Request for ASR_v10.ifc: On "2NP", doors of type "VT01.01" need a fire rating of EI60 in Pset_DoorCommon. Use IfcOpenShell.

First a look at what the model holds.

```python
import ifcopenshell
import ifcopenshell.util.element

model = ifcopenshell.open("ASR_v10.ifc")
print(model.schema)
storey = next(s for s in model.by_type("IfcBuildingStorey") if s.Name == "2NP")
doors = [e for e in ifcopenshell.util.element.get_decomposition(storey) if e.is_a("IfcDoor")]
seen = {}
for e in doors:
    element_type = ifcopenshell.util.element.get_type(e)
    key = (element_type.Name if element_type != e and element_type else None, ifcopenshell.util.element.get_pset(e, "Pset_DoorCommon", "FireRating"))
    seen[key] = seen.get(key, 0) + 1
for (name, value), count in sorted(seen.items(), key=str):
    print(count, "x", name, "|", value)
```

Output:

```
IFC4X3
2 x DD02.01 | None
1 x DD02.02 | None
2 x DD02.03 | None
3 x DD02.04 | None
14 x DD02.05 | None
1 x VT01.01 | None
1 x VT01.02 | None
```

```python
import ifcopenshell
import ifcopenshell.api.pset
import ifcopenshell.util.element

model = ifcopenshell.open("ASR_v10.ifc")

storey = next(s for s in model.by_type("IfcBuildingStorey") if s.Name == "2NP")
doors = [e for e in ifcopenshell.util.element.get_decomposition(storey) if e.is_a("IfcDoor")]

count = 0
for e in doors:
    element_type = ifcopenshell.util.element.get_type(e)
    if element_type in (None, e) or element_type.Name != "VT01.01":
        continue
    # add_pset returns the element's existing set when there is one.
    pset = ifcopenshell.api.pset.add_pset(model, product=e, name="Pset_DoorCommon")
    ifcopenshell.api.pset.edit_pset(model, pset=pset, properties={"FireRating": "EI60"})
    count += 1

print(count, "doors updated")

model.write("ASR_v10_rev.ifc")
```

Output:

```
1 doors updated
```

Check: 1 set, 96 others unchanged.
